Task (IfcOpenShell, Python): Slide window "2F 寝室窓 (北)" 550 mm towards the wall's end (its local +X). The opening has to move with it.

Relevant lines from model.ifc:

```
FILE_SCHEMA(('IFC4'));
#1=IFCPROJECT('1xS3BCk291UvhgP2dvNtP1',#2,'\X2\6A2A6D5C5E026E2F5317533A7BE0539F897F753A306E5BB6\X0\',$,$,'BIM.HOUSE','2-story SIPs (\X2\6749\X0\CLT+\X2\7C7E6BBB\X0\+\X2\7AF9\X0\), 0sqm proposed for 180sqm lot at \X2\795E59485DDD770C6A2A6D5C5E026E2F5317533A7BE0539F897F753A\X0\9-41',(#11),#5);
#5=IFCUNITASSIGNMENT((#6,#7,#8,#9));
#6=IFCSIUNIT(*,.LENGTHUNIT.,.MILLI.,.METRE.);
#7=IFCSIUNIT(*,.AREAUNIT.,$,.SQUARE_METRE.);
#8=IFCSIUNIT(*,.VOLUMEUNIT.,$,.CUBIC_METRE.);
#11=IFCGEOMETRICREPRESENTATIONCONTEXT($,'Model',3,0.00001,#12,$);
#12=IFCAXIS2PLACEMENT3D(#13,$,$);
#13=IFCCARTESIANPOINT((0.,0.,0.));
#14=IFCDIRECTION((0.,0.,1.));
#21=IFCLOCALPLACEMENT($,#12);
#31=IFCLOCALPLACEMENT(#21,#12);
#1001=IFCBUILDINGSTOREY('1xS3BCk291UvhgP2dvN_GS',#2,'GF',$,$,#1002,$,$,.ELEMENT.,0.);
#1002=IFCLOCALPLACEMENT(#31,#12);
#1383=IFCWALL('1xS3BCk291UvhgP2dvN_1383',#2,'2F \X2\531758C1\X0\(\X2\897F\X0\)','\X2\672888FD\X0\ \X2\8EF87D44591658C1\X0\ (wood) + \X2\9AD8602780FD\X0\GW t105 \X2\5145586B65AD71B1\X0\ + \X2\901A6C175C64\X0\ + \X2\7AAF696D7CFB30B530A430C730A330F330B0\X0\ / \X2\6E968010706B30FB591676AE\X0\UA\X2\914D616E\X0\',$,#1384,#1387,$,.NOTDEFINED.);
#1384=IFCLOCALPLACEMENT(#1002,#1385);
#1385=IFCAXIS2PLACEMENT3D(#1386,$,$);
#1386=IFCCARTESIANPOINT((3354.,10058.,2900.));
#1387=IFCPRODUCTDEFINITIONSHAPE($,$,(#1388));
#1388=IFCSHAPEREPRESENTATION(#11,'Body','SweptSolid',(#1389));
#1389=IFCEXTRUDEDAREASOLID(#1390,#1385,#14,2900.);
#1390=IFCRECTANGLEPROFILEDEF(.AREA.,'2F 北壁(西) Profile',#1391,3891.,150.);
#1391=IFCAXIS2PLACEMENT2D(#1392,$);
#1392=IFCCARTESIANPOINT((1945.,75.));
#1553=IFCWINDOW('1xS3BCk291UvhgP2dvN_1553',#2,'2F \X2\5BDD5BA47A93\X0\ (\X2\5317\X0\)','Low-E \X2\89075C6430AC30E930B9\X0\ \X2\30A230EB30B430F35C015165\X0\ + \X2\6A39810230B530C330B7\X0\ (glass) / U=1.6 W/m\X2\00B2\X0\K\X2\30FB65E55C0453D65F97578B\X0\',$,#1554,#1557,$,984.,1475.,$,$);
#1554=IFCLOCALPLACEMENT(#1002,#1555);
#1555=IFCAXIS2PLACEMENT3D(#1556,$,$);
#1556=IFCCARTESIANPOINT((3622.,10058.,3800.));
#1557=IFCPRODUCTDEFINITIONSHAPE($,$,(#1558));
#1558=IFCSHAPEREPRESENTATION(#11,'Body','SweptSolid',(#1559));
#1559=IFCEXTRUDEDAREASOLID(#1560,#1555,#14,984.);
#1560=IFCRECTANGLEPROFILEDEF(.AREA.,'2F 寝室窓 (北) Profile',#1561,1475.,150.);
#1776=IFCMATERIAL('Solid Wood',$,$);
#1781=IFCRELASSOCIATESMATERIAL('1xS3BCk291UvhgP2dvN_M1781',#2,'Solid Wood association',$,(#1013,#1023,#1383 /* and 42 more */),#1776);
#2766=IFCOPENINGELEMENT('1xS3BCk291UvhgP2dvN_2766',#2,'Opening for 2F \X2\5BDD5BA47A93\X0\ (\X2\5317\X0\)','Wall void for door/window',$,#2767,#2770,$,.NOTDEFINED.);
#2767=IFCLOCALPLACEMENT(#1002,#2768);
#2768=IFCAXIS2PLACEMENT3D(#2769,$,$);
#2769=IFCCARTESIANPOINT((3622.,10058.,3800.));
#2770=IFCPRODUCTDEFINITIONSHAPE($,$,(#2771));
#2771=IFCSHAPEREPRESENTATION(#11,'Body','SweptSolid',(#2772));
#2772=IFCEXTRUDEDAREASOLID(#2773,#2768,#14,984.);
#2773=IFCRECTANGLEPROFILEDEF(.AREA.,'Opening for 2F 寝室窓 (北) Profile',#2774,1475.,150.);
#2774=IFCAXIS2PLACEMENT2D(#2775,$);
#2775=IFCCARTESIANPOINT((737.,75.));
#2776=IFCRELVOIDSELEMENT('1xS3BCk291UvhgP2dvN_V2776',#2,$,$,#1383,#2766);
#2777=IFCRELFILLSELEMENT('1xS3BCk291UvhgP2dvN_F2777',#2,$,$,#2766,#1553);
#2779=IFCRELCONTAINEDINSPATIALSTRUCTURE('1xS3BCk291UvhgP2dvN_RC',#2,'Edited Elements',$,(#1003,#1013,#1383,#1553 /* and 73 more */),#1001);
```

```python
import ifcopenshell
import ifcopenshell.api.geometry
import ifcopenshell.util.placement
import ifcopenshell.util.unit

model = ifcopenshell.open("model.ifc")
unit_scale = ifcopenshell.util.unit.calculate_unit_scale(model)

window = model.by_guid("1xS3BCk291UvhgP2dvN_1553")
opening = window.FillsVoids[0].RelatingOpeningElement
wall = opening.VoidsElements[0].RelatingBuildingElement

wall_matrix = ifcopenshell.util.placement.get_local_placement(wall.ObjectPlacement)
shift = wall_matrix[:3, 0] * 0.55 / unit_scale
before = ifcopenshell.util.placement.get_local_placement(window.ObjectPlacement)[:3, 3].copy()

# The window is not placed relative to its opening, so move both.
for product in (opening, window):
    matrix = ifcopenshell.util.placement.get_local_placement(product.ObjectPlacement)
    matrix[:3, 3] += shift
    ifcopenshell.api.geometry.edit_object_placement(model, product=product, matrix=matrix, is_si=False)

after = ifcopenshell.util.placement.get_local_placement(window.ObjectPlacement)[:3, 3]
print("window moved by", (after - before).round(3) + 0.0)

model.write("model_edited.ifc")
```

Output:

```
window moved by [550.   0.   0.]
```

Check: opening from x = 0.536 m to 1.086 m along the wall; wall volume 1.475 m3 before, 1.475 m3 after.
